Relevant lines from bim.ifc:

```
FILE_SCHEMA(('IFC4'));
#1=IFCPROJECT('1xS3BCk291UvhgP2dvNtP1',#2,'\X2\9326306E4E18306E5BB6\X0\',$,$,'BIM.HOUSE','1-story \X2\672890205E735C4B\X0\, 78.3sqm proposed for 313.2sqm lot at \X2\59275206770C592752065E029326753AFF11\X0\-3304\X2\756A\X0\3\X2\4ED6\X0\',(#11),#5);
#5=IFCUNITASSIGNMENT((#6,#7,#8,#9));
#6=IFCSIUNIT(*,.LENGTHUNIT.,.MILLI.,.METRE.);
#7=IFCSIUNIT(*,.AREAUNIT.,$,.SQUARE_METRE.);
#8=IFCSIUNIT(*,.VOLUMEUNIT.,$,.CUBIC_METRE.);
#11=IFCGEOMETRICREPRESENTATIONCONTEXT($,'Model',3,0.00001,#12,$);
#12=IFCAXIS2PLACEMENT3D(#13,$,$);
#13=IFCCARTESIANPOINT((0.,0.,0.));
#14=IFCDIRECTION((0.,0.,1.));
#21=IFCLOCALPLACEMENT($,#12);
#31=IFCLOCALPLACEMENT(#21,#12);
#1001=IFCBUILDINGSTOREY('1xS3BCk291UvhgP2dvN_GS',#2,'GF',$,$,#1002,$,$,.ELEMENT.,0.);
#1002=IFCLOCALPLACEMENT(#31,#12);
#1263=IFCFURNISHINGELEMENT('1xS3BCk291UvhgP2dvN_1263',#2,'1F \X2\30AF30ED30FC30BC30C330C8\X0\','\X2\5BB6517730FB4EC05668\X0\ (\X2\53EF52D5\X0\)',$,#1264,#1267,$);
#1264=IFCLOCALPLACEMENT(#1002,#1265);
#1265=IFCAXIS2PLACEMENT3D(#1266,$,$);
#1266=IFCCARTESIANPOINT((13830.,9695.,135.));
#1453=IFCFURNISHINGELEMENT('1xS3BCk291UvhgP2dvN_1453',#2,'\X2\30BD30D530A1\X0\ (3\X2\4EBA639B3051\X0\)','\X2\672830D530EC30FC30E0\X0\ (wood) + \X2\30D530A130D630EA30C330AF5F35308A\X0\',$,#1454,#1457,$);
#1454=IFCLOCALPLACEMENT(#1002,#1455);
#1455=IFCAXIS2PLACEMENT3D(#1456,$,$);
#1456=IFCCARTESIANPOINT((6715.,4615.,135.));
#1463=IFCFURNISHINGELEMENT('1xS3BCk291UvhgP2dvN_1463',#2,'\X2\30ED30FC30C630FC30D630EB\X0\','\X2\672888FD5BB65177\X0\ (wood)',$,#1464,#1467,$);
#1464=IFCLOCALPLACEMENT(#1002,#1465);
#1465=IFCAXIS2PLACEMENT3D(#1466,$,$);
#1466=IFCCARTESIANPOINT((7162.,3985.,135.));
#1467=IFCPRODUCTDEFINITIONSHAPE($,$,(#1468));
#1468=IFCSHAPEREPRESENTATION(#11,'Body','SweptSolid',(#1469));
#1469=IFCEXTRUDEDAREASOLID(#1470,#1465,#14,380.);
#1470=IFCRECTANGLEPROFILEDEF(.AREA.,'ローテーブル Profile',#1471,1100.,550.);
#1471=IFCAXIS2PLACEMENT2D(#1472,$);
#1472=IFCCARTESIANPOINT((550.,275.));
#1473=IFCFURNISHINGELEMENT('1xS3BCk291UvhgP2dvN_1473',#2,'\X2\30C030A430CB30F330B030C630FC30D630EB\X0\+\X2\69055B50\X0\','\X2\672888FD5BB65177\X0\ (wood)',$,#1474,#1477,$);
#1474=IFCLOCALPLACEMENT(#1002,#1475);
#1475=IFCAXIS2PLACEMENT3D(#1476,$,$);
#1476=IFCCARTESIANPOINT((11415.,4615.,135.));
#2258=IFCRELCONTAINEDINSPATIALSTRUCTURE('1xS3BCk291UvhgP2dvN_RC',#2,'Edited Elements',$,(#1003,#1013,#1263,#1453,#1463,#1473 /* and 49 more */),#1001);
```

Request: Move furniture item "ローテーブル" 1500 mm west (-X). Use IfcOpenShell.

```python
import ifcopenshell
import ifcopenshell.api.geometry
import ifcopenshell.util.placement
import ifcopenshell.util.unit

model = ifcopenshell.open("bim.ifc")
unit_scale = ifcopenshell.util.unit.calculate_unit_scale(model)

item = model.by_guid("1xS3BCk291UvhgP2dvN_1463")
matrix = ifcopenshell.util.placement.get_local_placement(item.ObjectPlacement)
matrix[0, 3] -= 1.5 / unit_scale
ifcopenshell.api.geometry.edit_object_placement(model, product=item, matrix=matrix, is_si=False)

print(ifcopenshell.util.placement.get_local_placement(item.ObjectPlacement).round(3) + 0.0)

model.write("bim_updated.ifc")
```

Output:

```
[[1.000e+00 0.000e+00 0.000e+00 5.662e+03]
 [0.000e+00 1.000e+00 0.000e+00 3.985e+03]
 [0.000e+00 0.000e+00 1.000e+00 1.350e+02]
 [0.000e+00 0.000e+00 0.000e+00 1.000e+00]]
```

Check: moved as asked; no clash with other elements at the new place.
